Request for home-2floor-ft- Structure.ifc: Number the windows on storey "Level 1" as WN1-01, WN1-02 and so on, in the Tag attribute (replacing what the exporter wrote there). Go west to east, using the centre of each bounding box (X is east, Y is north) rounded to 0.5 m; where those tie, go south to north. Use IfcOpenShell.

First a look at what the model holds.

```python
import ifcopenshell
import ifcopenshell.util.element
import ifcopenshell.util.placement

model = ifcopenshell.open("home-2floor-ft- Structure.ifc")
print(model.schema)
storey = next(s for s in model.by_type("IfcBuildingStorey") if s.Name == "Level 1")
windows = [e for e in ifcopenshell.util.element.get_decomposition(storey) if e.is_a("IfcWindow")]
for e in sorted(windows, key=lambda e: e.id()):
    origin = ifcopenshell.util.placement.get_local_placement(e.ObjectPlacement)[:3, 3]
    print(e.id(), e.Tag, e.Name, origin.round(2) + 0.0, sep=" | ")
```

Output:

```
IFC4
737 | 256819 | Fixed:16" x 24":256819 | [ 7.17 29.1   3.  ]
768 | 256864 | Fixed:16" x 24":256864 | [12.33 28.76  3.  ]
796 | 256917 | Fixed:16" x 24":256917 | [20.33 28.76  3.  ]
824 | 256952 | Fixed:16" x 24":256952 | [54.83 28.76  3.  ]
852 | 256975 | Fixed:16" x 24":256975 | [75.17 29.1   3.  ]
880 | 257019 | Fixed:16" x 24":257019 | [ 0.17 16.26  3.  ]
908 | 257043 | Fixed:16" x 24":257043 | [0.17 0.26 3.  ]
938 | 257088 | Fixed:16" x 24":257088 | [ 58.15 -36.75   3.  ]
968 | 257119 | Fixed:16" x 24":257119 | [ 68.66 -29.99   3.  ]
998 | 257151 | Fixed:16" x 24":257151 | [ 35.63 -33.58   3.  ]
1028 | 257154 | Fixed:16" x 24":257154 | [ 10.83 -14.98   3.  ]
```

```python
import ifcopenshell
import ifcopenshell.geom
import ifcopenshell.util.element
import ifcopenshell.util.shape

model = ifcopenshell.open("home-2floor-ft- Structure.ifc")
settings = ifcopenshell.geom.settings()
settings.set("use-world-coords", True)


def centre(element):
    shape = ifcopenshell.geom.create_shape(settings, element)
    return ifcopenshell.util.shape.get_bbox_centroid(shape.geometry)


storey = next(s for s in model.by_type("IfcBuildingStorey") if s.Name == "Level 1")
windows = [e for e in ifcopenshell.util.element.get_decomposition(storey) if e.is_a("IfcWindow")]

# Insertion points can sit at a corner or the storey origin, so sort by the geometry (in metres).
centres = {e: centre(e) for e in windows}
windows.sort(key=lambda e: (round(centres[e][0] / 0.5), centres[e][1]))

for i, e in enumerate(windows, start=1):
    number = f"WN1-{i:02d}"
    e.Tag = number
    print(e.id(), number)

model.write("home-2floor-ft- Structure_edited.ifc")
```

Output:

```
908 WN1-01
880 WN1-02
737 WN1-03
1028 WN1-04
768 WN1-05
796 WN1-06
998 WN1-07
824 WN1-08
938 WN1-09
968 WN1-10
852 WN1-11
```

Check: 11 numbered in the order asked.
